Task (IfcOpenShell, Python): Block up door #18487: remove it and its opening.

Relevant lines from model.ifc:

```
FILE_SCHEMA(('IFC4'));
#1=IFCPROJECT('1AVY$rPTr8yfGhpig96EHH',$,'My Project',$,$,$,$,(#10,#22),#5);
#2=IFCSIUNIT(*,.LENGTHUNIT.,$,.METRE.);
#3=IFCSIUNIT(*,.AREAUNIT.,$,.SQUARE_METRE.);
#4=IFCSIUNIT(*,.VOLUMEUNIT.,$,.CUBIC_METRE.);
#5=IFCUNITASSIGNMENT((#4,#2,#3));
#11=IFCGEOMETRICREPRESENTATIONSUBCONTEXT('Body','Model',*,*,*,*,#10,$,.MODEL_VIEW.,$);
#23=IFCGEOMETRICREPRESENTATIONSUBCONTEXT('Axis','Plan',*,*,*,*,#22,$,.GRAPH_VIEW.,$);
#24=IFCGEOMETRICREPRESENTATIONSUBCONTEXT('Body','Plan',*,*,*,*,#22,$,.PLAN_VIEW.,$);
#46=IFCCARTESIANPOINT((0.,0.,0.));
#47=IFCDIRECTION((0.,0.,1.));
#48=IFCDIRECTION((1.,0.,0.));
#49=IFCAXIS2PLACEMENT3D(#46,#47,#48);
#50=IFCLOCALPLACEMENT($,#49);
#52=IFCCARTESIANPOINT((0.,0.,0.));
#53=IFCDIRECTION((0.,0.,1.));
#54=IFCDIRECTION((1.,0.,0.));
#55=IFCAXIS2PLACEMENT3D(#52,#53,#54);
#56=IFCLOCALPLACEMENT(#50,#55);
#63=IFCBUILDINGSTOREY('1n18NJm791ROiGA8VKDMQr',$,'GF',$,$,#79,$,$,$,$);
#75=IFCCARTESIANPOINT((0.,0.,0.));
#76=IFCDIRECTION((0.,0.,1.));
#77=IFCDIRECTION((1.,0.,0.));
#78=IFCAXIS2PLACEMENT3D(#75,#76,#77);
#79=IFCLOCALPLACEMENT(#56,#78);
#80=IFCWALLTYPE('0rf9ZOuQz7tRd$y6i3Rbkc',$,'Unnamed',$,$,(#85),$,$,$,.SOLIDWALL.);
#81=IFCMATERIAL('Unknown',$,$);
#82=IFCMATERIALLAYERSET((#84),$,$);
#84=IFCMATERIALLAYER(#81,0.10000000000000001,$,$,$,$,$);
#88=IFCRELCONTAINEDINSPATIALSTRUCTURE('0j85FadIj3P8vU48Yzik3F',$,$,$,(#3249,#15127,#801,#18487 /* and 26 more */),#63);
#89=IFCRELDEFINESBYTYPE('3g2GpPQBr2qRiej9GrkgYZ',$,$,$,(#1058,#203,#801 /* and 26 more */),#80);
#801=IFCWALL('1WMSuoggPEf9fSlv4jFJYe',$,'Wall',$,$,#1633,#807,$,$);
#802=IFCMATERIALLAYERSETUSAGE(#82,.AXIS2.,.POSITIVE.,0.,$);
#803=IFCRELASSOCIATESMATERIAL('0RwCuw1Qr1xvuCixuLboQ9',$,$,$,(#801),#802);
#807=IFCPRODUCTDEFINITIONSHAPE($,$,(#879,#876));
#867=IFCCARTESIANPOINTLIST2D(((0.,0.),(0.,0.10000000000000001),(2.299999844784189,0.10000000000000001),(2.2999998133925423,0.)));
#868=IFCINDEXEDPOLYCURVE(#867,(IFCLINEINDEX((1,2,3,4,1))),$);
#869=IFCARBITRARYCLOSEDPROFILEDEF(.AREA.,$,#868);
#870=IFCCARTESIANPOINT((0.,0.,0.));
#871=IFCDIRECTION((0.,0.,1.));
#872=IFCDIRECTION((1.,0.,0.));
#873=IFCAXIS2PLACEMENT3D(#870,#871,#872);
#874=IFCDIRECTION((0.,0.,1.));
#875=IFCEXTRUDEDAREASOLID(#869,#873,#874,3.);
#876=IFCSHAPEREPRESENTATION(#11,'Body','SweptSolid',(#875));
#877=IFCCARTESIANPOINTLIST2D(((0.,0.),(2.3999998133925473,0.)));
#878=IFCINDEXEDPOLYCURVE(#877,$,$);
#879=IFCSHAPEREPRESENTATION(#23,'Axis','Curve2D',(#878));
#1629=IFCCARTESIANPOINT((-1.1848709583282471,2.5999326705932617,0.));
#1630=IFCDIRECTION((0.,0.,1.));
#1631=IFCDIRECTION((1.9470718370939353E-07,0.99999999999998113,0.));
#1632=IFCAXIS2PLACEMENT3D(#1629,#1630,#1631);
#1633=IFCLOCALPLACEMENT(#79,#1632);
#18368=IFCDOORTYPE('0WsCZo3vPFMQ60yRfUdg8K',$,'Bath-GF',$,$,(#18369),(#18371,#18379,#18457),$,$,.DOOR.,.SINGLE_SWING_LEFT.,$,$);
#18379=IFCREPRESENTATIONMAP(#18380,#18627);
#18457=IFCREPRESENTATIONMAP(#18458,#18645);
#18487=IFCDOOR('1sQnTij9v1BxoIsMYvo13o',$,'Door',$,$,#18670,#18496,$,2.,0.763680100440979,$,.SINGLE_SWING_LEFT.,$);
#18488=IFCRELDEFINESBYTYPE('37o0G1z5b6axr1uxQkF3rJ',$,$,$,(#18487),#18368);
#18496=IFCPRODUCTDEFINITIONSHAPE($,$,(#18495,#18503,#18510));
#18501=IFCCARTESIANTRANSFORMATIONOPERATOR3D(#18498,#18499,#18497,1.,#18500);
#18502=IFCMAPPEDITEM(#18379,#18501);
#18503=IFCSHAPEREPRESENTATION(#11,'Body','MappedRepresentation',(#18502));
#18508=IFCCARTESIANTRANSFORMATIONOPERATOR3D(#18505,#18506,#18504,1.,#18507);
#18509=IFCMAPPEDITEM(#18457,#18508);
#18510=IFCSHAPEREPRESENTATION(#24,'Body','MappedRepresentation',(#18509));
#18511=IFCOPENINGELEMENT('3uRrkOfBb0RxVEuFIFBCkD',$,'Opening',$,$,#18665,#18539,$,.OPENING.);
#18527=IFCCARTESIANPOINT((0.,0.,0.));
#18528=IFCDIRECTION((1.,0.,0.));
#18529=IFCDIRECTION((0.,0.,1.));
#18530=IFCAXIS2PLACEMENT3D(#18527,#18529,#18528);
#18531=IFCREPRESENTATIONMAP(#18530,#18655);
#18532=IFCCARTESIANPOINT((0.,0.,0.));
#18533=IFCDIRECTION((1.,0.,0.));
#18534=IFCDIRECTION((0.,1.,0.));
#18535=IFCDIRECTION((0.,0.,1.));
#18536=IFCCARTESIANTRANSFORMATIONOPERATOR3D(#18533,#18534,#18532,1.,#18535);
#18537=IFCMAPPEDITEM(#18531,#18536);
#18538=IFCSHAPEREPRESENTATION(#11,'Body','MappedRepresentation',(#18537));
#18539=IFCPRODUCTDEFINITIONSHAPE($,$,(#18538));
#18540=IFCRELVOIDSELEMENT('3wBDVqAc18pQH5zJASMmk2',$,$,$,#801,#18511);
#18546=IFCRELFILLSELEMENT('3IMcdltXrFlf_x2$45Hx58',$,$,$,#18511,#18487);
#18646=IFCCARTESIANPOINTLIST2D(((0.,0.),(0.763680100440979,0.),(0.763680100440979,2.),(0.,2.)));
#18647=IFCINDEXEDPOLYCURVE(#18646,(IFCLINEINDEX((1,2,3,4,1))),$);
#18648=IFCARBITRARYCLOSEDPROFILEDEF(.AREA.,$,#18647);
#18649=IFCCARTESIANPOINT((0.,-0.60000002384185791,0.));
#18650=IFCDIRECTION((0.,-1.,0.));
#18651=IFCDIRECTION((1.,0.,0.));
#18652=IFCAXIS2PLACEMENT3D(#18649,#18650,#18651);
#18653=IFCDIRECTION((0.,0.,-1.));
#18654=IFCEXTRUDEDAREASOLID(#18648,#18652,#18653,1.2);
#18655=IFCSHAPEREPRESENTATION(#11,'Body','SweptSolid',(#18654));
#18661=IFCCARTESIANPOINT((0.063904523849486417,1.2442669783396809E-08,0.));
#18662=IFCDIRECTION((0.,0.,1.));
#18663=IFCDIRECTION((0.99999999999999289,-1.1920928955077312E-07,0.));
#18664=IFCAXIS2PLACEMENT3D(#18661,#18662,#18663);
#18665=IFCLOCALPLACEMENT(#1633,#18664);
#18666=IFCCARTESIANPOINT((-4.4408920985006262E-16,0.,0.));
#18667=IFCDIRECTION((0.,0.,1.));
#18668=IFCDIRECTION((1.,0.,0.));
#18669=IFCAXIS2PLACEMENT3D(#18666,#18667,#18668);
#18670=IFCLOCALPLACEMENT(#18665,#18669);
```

```python
import ifcopenshell
import ifcopenshell.api.feature
import ifcopenshell.api.root
import ifcopenshell.geom
import ifcopenshell.util.shape

model = ifcopenshell.open("model.ifc")
settings = ifcopenshell.geom.settings()


def volume(element):
    """Net volume in cubic metres, openings subtracted."""
    shape = ifcopenshell.geom.create_shape(settings, element)
    return ifcopenshell.util.shape.get_volume(shape.geometry)


door = model.by_guid("1sQnTij9v1BxoIsMYvo13o")
opening = door.FillsVoids[0].RelatingOpeningElement
wall = opening.VoidsElements[0].RelatingBuildingElement
before = volume(wall)

ifcopenshell.api.root.remove_product(model, product=door)
ifcopenshell.api.feature.remove_feature(model, feature=opening)

after = volume(wall)

print(f"wall volume {before:.3f} -> {after:.3f} m3")

model.write("model_v2.ifc")
```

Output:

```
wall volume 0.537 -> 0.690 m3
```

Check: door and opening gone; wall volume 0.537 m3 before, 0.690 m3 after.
